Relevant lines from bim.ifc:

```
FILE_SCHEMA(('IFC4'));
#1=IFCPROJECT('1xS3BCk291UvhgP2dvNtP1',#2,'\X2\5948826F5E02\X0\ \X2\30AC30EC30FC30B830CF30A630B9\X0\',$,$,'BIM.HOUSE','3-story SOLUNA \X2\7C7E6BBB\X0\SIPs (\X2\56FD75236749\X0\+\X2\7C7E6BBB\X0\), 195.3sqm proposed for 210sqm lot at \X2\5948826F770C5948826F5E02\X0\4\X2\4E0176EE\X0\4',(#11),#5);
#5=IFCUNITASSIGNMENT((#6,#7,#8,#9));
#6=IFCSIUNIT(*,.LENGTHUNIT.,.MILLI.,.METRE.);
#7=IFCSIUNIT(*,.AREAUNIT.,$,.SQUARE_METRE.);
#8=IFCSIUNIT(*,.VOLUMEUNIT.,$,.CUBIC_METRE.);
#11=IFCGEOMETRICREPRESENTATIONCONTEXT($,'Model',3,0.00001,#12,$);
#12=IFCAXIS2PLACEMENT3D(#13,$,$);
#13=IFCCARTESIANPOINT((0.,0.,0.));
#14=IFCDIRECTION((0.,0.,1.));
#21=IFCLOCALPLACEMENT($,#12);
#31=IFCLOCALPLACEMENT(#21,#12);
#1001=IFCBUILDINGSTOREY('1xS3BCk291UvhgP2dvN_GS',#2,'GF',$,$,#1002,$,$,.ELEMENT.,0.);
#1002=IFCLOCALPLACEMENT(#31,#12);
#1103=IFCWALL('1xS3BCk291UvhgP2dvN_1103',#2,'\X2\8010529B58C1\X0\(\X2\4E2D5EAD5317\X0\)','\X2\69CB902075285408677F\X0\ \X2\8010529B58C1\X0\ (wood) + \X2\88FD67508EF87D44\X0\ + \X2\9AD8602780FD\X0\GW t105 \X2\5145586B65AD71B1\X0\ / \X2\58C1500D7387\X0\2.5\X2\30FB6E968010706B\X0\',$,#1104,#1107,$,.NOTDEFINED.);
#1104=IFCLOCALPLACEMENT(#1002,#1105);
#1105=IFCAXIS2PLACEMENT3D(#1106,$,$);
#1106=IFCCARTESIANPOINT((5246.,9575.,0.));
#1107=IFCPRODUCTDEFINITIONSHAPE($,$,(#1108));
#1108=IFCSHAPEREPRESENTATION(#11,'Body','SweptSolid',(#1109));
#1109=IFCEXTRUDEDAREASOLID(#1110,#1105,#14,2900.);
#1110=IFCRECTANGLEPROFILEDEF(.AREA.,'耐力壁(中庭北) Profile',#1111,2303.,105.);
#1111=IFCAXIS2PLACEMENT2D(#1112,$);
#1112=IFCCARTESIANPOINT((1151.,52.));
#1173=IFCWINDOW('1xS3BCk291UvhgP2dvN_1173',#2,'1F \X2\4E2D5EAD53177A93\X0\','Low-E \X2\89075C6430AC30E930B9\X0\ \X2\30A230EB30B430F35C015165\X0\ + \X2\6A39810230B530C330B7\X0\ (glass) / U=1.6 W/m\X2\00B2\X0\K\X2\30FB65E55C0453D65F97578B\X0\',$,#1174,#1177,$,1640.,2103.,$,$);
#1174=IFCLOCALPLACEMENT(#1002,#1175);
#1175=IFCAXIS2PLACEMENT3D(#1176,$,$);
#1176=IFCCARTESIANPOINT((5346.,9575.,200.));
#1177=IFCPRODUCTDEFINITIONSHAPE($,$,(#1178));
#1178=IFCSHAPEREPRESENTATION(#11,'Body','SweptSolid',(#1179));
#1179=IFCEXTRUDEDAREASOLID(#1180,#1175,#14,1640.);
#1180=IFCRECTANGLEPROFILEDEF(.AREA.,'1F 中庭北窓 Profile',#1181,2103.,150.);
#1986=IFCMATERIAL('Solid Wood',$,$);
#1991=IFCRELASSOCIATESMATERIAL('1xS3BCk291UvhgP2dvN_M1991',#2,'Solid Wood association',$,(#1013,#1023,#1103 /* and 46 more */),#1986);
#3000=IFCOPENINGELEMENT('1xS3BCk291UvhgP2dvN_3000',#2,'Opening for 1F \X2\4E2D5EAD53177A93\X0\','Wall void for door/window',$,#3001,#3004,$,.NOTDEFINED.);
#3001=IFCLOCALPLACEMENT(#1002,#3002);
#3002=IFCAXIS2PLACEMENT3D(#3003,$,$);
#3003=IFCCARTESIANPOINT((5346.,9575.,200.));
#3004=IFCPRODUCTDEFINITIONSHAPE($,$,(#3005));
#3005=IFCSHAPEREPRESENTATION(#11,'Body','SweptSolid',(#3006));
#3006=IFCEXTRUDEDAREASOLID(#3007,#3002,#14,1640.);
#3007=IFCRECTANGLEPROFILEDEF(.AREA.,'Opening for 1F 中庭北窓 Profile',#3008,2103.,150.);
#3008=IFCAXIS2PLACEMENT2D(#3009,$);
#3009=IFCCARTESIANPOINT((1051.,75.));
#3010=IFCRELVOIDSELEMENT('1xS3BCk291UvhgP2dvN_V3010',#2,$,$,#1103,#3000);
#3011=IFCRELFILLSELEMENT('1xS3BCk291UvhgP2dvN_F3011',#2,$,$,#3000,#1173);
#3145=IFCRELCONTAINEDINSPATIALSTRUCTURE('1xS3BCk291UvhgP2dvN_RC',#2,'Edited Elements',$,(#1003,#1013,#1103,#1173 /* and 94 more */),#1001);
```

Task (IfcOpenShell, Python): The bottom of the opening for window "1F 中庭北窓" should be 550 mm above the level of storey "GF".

```python
import numpy as np
import ifcopenshell
import ifcopenshell.api.geometry
import ifcopenshell.geom
import ifcopenshell.util.element
import ifcopenshell.util.placement
import ifcopenshell.util.shape
import ifcopenshell.util.unit

model = ifcopenshell.open("bim.ifc")
unit_scale = ifcopenshell.util.unit.calculate_unit_scale(model)

window = model.by_id(1173)
opening = window.FillsVoids[0].RelatingOpeningElement
storey = ifcopenshell.util.element.get_container(window, ifc_class="IfcBuildingStorey")
level = ifcopenshell.util.placement.get_local_placement(storey.ObjectPlacement)[2, 3]

# The opening's origin need not be at the sill, so measure its lowest point.
shape = ifcopenshell.geom.create_shape(ifcopenshell.geom.settings(), opening)
bottom = ifcopenshell.util.shape.get_shape_bottom_elevation(shape, shape.geometry) / unit_scale
dz = level + 0.55 / unit_scale - bottom

shift = np.array([0.0, 0.0, dz])
# The window is not placed relative to its opening, so move both.
for product in (opening, window):
    matrix = ifcopenshell.util.placement.get_local_placement(product.ObjectPlacement)
    matrix[:3, 3] += shift
    ifcopenshell.api.geometry.edit_object_placement(model, product=product, matrix=matrix, is_si=False)

print(f"moved by {dz * unit_scale:+.3f} m")

model.write("bim_rev.ifc")
```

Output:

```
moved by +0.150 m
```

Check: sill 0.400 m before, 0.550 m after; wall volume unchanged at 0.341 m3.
